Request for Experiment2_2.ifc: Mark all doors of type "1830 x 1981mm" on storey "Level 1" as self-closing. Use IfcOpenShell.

First a look at what the model holds.

```python
import ifcopenshell
import ifcopenshell.util.element

model = ifcopenshell.open("Experiment2_2.ifc")
print(model.schema)
storey = next(s for s in model.by_type("IfcBuildingStorey") if s.Name == "Level 1")
doors = [e for e in ifcopenshell.util.element.get_decomposition(storey) if e.is_a("IfcDoor")]
seen = {}
for e in doors:
    element_type = ifcopenshell.util.element.get_type(e)
    key = (element_type.Name if element_type != e and element_type else None, ifcopenshell.util.element.get_pset(e, "Pset_DoorCommon", "SelfClosing"))
    seen[key] = seen.get(key, 0) + 1
for (name, value), count in sorted(seen.items(), key=str):
    print(count, "x", name, "|", value)
```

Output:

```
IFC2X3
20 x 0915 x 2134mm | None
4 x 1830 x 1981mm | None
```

```python
import ifcopenshell
import ifcopenshell.api.pset
import ifcopenshell.util.element

model = ifcopenshell.open("Experiment2_2.ifc")

storey = next(s for s in model.by_type("IfcBuildingStorey") if s.Name == "Level 1")
doors = [e for e in ifcopenshell.util.element.get_decomposition(storey) if e.is_a("IfcDoor")]

count = 0
for e in doors:
    element_type = ifcopenshell.util.element.get_type(e)
    if element_type in (None, e) or element_type.Name != "1830 x 1981mm":
        continue
    # add_pset returns the element's existing set when there is one.
    pset = ifcopenshell.api.pset.add_pset(model, product=e, name="Pset_DoorCommon")
    ifcopenshell.api.pset.edit_pset(model, pset=pset, properties={"SelfClosing": True})
    count += 1

print(count, "doors updated")

model.write("Experiment2_2_rev.ifc")
```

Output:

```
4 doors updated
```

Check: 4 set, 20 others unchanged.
